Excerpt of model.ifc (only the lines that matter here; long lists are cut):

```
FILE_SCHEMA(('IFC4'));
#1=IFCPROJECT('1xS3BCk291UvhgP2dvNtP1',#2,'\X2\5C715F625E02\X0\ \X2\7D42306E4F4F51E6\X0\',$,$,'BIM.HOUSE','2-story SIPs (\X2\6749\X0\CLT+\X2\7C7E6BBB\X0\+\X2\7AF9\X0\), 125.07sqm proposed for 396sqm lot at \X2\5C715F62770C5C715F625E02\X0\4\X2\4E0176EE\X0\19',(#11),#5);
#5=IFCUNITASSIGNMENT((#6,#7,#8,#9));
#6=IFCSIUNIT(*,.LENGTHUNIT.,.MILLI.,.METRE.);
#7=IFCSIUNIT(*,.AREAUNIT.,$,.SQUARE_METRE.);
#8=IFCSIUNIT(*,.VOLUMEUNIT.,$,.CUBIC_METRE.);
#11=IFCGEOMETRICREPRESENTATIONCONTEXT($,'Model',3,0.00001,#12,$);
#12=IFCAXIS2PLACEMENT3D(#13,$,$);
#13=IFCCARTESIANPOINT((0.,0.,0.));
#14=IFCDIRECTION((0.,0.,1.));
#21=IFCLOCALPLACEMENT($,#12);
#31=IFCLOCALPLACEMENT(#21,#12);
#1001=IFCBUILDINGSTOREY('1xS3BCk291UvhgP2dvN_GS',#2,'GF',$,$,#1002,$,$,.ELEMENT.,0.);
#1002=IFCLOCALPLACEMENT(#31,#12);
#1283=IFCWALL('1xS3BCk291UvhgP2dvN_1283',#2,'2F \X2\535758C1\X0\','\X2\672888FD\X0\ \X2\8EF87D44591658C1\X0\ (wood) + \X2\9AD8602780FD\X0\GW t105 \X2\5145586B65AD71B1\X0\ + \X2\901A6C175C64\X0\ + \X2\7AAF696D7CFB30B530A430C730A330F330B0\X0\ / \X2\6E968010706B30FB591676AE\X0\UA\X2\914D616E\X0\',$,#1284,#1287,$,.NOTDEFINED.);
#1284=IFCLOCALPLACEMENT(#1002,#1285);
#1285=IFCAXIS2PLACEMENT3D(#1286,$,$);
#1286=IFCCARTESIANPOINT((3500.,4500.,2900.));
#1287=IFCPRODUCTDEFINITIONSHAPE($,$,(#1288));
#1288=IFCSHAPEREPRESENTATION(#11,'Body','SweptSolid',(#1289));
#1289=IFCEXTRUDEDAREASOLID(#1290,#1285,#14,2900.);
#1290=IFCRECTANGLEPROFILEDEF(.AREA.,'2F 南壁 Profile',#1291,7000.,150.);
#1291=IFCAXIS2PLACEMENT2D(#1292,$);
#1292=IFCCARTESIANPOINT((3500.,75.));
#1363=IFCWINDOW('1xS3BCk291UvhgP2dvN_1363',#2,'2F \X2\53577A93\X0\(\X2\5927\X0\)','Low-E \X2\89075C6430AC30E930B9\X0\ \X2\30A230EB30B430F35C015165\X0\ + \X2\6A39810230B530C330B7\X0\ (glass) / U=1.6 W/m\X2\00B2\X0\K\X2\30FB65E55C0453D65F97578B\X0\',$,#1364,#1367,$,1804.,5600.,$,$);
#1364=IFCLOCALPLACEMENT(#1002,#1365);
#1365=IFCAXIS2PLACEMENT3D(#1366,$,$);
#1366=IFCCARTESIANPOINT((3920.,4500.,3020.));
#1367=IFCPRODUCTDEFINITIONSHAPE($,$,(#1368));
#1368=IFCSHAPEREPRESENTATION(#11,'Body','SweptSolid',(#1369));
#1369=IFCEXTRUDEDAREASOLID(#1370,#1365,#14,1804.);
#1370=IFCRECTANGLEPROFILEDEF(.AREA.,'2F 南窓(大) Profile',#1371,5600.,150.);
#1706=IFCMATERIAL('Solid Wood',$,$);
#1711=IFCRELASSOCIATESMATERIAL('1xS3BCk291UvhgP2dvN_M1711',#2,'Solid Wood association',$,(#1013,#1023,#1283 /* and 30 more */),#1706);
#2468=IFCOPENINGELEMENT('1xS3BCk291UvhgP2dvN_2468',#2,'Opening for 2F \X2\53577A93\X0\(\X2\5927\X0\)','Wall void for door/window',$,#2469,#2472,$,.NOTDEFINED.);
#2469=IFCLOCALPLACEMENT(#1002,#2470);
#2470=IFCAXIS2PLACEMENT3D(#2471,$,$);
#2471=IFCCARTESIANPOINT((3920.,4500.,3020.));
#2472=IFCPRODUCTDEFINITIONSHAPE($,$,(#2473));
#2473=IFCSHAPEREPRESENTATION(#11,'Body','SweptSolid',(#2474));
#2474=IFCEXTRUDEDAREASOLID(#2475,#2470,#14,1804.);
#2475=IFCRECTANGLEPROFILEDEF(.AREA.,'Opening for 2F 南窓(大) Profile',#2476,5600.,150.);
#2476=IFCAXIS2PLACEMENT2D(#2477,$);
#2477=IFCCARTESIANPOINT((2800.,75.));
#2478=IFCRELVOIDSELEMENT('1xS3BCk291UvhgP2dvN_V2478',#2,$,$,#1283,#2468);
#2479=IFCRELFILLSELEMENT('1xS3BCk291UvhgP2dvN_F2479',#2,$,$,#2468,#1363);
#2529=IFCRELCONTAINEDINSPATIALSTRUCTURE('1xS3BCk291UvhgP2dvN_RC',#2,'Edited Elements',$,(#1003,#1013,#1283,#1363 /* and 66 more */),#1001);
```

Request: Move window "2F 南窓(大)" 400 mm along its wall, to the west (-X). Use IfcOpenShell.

```python
import ifcopenshell
import ifcopenshell.api.geometry
import ifcopenshell.util.placement

model = ifcopenshell.open("model.ifc")

window = model.by_guid("1xS3BCk291UvhgP2dvN_1363")
opening = window.FillsVoids[0].RelatingOpeningElement
wall = opening.VoidsElements[0].RelatingBuildingElement

wall_matrix = ifcopenshell.util.placement.get_local_placement(wall.ObjectPlacement)
shift = wall_matrix[:3, 0] * -400.0
before = ifcopenshell.util.placement.get_local_placement(window.ObjectPlacement)[:3, 3].copy()

# The window is not placed relative to its opening, so move both.
for product in (opening, window):
    matrix = ifcopenshell.util.placement.get_local_placement(product.ObjectPlacement)
    matrix[:3, 3] += shift
    ifcopenshell.api.geometry.edit_object_placement(model, product=product, matrix=matrix, is_si=False)

after = ifcopenshell.util.placement.get_local_placement(window.ObjectPlacement)[:3, 3]
print("window moved by", (after - before).round(3) + 0.0)

model.write("model_updated.ifc")
```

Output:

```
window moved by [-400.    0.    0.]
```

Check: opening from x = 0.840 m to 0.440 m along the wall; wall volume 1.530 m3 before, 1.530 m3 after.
